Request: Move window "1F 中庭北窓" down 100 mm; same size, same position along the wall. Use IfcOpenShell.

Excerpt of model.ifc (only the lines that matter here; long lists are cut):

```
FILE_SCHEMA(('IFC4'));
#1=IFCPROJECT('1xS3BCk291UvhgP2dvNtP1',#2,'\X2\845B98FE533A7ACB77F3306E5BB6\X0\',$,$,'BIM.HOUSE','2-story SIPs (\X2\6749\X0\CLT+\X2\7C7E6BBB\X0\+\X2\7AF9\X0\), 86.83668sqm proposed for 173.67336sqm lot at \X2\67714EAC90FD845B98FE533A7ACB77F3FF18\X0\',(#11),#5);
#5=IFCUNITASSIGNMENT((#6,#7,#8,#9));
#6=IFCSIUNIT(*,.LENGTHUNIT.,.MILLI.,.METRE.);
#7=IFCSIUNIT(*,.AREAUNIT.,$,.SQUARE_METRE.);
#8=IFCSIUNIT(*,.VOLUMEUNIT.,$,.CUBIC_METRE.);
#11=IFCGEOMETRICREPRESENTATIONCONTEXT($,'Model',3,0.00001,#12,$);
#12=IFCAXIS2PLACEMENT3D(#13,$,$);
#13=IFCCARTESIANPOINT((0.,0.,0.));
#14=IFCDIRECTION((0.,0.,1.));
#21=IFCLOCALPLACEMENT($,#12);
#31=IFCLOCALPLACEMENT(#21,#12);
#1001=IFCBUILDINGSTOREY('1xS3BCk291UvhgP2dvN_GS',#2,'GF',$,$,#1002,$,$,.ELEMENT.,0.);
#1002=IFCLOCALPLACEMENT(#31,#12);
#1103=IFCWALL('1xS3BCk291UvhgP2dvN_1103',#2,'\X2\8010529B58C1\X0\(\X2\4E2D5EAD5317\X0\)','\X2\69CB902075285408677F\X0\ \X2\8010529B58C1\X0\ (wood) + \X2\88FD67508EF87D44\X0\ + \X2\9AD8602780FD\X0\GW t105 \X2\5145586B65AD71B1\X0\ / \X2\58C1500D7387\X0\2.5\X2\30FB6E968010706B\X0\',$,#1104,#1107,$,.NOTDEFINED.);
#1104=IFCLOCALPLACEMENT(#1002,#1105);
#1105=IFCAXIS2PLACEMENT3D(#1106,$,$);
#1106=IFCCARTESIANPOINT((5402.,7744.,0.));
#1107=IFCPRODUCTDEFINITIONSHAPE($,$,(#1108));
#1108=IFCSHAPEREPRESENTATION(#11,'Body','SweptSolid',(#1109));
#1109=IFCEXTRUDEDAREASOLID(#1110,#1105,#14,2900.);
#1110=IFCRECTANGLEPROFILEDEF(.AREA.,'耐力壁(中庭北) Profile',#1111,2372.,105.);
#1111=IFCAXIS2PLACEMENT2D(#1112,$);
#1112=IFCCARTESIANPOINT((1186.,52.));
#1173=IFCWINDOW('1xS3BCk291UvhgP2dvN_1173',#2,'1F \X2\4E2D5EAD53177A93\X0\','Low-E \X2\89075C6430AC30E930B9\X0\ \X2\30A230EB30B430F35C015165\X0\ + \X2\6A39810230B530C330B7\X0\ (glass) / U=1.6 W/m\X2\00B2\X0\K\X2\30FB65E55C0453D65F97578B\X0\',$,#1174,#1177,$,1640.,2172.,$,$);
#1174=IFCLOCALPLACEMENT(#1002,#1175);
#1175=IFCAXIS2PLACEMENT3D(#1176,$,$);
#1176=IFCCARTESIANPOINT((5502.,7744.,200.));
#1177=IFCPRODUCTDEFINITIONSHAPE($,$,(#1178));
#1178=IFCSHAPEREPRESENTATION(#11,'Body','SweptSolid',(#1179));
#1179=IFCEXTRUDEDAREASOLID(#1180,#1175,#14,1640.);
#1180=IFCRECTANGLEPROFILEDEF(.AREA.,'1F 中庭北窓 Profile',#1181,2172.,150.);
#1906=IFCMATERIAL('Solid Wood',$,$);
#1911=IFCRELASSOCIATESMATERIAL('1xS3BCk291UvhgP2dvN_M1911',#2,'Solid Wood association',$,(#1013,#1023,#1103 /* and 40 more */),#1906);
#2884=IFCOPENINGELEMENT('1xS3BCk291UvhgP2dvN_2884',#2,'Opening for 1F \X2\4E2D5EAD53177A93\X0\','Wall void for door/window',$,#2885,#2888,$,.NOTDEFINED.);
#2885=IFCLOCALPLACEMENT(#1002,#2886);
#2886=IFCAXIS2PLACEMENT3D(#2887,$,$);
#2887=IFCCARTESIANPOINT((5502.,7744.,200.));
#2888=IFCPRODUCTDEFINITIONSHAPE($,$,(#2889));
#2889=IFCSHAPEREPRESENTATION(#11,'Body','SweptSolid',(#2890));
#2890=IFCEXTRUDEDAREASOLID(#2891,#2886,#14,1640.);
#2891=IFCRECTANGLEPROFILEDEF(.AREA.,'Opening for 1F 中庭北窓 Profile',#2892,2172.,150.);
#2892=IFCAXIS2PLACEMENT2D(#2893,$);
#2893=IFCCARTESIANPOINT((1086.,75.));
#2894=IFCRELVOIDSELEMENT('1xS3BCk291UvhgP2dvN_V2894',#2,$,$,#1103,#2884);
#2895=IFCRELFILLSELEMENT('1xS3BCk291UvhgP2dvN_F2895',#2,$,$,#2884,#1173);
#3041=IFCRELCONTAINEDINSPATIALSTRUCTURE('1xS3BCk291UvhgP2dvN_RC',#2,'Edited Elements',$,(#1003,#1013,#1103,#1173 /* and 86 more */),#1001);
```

```python
import numpy as np
import ifcopenshell
import ifcopenshell.api.geometry
import ifcopenshell.util.placement
import ifcopenshell.util.unit

model = ifcopenshell.open("model.ifc")
unit_scale = ifcopenshell.util.unit.calculate_unit_scale(model)

window = model.by_guid("1xS3BCk291UvhgP2dvN_1173")
opening = window.FillsVoids[0].RelatingOpeningElement
dz = -0.1 / unit_scale

shift = np.array([0.0, 0.0, dz])
# The window is not placed relative to its opening, so move both.
for product in (opening, window):
    matrix = ifcopenshell.util.placement.get_local_placement(product.ObjectPlacement)
    matrix[:3, 3] += shift
    ifcopenshell.api.geometry.edit_object_placement(model, product=product, matrix=matrix, is_si=False)

print(f"moved by {dz * unit_scale:+.3f} m")

model.write("model_rev.ifc")
```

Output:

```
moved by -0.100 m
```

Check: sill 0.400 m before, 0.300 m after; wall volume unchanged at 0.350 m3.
